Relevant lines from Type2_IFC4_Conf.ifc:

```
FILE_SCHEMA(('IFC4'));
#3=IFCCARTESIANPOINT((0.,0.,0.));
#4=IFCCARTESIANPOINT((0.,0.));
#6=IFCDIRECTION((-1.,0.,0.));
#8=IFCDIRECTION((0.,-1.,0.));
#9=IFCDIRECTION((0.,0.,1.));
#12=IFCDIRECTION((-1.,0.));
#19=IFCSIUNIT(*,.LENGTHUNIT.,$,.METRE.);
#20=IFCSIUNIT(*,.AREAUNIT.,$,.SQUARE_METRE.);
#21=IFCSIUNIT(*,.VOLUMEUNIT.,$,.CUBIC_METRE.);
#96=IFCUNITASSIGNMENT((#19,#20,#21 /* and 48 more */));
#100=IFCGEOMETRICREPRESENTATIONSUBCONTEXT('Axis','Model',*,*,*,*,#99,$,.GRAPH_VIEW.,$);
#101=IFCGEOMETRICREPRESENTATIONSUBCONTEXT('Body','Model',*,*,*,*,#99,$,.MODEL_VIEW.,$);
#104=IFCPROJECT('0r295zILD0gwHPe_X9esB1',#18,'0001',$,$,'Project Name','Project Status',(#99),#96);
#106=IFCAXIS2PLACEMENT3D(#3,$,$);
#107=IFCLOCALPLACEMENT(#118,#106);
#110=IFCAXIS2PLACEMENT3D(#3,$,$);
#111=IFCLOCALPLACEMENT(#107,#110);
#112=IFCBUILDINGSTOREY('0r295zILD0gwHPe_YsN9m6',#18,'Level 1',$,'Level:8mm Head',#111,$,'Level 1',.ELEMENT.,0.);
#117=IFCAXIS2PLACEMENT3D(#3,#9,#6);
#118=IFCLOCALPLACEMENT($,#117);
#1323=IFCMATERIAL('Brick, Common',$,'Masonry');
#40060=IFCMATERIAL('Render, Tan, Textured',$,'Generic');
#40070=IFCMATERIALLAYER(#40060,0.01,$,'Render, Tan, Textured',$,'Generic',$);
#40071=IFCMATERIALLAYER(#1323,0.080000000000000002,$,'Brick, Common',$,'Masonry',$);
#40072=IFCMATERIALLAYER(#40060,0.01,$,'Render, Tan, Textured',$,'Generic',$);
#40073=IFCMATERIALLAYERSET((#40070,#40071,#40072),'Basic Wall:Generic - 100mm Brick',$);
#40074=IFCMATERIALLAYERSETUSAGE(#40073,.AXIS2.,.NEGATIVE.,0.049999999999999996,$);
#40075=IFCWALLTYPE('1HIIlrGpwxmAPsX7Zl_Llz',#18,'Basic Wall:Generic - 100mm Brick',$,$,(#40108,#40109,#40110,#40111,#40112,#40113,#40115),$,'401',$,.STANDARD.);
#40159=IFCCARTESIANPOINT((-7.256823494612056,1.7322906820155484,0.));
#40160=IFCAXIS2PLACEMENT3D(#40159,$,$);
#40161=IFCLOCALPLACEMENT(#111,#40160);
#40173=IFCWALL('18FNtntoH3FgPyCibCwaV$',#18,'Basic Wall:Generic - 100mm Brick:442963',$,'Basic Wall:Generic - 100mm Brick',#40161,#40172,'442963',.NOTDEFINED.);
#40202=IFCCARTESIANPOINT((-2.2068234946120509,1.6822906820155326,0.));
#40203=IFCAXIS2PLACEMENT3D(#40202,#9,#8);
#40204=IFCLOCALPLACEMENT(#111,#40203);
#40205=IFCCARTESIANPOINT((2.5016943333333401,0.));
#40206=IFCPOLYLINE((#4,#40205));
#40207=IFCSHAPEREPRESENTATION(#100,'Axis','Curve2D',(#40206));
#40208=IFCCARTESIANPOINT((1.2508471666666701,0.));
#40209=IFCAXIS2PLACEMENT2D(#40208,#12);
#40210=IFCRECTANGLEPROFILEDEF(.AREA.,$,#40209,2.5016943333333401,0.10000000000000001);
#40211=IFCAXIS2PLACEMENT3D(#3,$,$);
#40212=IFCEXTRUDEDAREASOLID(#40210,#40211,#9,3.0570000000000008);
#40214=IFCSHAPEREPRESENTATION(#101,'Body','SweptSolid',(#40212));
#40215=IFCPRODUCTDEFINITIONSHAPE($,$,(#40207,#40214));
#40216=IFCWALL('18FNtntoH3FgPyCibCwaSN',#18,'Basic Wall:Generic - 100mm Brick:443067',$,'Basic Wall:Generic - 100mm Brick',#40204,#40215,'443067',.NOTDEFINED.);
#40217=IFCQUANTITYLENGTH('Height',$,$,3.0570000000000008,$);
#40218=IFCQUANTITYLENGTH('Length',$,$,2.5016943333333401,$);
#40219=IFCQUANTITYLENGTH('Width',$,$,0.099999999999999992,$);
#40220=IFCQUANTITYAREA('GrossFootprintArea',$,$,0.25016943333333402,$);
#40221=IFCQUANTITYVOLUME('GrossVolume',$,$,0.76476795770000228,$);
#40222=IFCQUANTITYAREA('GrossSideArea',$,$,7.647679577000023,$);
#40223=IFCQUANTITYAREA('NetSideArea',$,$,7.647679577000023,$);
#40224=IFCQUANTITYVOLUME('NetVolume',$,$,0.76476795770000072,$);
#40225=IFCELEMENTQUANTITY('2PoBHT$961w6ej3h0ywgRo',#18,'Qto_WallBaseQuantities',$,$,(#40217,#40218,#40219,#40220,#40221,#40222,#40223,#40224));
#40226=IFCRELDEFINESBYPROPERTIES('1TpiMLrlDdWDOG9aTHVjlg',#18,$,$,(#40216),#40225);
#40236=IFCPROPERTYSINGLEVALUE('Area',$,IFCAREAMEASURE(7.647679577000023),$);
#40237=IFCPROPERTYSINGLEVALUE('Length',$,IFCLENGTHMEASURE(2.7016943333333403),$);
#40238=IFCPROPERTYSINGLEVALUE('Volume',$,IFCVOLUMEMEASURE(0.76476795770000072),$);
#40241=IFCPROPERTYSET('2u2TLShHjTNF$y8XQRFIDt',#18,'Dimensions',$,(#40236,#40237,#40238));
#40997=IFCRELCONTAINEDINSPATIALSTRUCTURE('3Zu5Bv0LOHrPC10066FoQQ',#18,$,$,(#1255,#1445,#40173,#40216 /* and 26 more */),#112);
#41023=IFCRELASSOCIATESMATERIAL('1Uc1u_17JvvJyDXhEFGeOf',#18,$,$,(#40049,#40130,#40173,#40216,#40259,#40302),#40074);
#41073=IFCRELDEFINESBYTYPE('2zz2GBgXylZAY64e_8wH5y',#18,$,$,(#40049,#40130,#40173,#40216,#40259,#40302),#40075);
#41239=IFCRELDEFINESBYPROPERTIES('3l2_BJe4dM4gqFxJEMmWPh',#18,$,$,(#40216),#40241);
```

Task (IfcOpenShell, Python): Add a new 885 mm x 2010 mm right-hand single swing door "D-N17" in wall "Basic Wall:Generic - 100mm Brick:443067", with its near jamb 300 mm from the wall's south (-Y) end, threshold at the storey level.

```python
import numpy as np
import ifcopenshell
import ifcopenshell.api.feature
import ifcopenshell.api.geometry
import ifcopenshell.api.pset
import ifcopenshell.api.root
import ifcopenshell.api.spatial
import ifcopenshell.geom
import ifcopenshell.util.element
import ifcopenshell.util.placement
import ifcopenshell.util.representation
import ifcopenshell.util.shape
import ifcopenshell.util.unit

model = ifcopenshell.open("Type2_IFC4_Conf.ifc")
unit_scale = ifcopenshell.util.unit.calculate_unit_scale(model)
area_scale = ifcopenshell.util.unit.calculate_unit_scale(model, "AREAUNIT")
volume_scale = ifcopenshell.util.unit.calculate_unit_scale(model, "VOLUMEUNIT")
settings = ifcopenshell.geom.settings()


def volume(element):
    """Net volume in cubic metres, openings subtracted."""
    shape = ifcopenshell.geom.create_shape(settings, element)
    return ifcopenshell.util.shape.get_volume(shape.geometry)


wall = model.by_guid("18FNtntoH3FgPyCibCwaSN")
storey = ifcopenshell.util.element.get_container(wall, ifc_class="IfcBuildingStorey")
context = ifcopenshell.util.representation.get_context(model, "Model", "Body", "MODEL_VIEW")
before = volume(wall)

width, height, from_end, sill = 0.885, 2.01, 0.3, 0.0  # metres

# The wall runs along its own X axis, and the end named is its -X end.
wall_shape = ifcopenshell.geom.create_shape(settings, wall)
x, y, z = ifcopenshell.util.shape.get_vertices(wall_shape.geometry).T
start = x.min() + from_end
face, thickness = float(y.min()), float(y.max() - y.min())
wall_matrix = ifcopenshell.util.placement.get_local_placement(wall.ObjectPlacement)
level = ifcopenshell.util.placement.get_local_placement(storey.ObjectPlacement)[2, 3]


def in_wall(x, y):
    """Placement at x, y metres in the wall's axes, at sill height."""
    matrix = wall_matrix.copy()
    matrix[:, 3] = wall_matrix @ np.array([x / unit_scale, y / unit_scale, 0.0, 1.0])
    matrix[2, 3] = level + sill / unit_scale
    return matrix


# Opening: a box that overshoots both wall faces by 50 mm.
opening = ifcopenshell.api.root.create_entity(model, ifc_class="IfcOpeningElement", predefined_type="OPENING")
box = ifcopenshell.api.geometry.add_wall_representation(
    model, context=context, length=width, height=height, thickness=thickness + 0.1
)
ifcopenshell.api.geometry.assign_representation(model, product=opening, representation=box)
ifcopenshell.api.geometry.edit_object_placement(model, product=opening, matrix=in_wall(start, face - 0.05), is_si=False)
ifcopenshell.api.feature.add_feature(model, feature=opening, element=wall)

door = ifcopenshell.api.root.create_entity(model, ifc_class="IfcDoor", name="D-N17", predefined_type="DOOR")
door.OverallWidth, door.OverallHeight = width / unit_scale, height / unit_scale
door.OperationType = "SINGLE_SWING_RIGHT"
body = ifcopenshell.api.geometry.add_door_representation(
    model,
    context=context,
    overall_width=door.OverallWidth,
    overall_height=door.OverallHeight,
    operation_type="SINGLE_SWING_RIGHT",
    lining_properties={"LiningDepth": thickness / unit_scale, "ThresholdDepth": thickness / unit_scale},
)
ifcopenshell.api.geometry.assign_representation(model, product=door, representation=body)
ifcopenshell.api.spatial.assign_container(model, products=[door], relating_structure=storey)
ifcopenshell.api.feature.add_filling(model, opening=opening, element=door)

# The lining spans the wall, so the door starts at the wall face.
ifcopenshell.api.geometry.edit_object_placement(model, product=door, matrix=in_wall(start, face), is_si=False)

after = volume(wall)

# Update the wall's stored quantities.
qto = model.by_id(ifcopenshell.util.element.get_pset(wall, "Qto_WallBaseQuantities", should_inherit=False)["id"])
ifcopenshell.api.pset.edit_qto(model, qto=qto, properties={
    "NetSideArea": after / thickness / area_scale,
    "NetVolume": after / volume_scale,
})
pset = model.by_id(ifcopenshell.util.element.get_pset(wall, "Dimensions", should_inherit=False)["id"])
ifcopenshell.api.pset.edit_pset(model, pset=pset, properties={
    "Area": model.create_entity("IfcAreaMeasure", after / thickness / area_scale),
    "Volume": model.create_entity("IfcVolumeMeasure", after / volume_scale),
})

print(f"wall volume {before:.3f} -> {after:.3f} m3")

model.write("Type2_IFC4_Conf-out.ifc")
```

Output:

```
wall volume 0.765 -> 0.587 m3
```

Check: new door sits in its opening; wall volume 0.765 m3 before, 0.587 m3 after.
